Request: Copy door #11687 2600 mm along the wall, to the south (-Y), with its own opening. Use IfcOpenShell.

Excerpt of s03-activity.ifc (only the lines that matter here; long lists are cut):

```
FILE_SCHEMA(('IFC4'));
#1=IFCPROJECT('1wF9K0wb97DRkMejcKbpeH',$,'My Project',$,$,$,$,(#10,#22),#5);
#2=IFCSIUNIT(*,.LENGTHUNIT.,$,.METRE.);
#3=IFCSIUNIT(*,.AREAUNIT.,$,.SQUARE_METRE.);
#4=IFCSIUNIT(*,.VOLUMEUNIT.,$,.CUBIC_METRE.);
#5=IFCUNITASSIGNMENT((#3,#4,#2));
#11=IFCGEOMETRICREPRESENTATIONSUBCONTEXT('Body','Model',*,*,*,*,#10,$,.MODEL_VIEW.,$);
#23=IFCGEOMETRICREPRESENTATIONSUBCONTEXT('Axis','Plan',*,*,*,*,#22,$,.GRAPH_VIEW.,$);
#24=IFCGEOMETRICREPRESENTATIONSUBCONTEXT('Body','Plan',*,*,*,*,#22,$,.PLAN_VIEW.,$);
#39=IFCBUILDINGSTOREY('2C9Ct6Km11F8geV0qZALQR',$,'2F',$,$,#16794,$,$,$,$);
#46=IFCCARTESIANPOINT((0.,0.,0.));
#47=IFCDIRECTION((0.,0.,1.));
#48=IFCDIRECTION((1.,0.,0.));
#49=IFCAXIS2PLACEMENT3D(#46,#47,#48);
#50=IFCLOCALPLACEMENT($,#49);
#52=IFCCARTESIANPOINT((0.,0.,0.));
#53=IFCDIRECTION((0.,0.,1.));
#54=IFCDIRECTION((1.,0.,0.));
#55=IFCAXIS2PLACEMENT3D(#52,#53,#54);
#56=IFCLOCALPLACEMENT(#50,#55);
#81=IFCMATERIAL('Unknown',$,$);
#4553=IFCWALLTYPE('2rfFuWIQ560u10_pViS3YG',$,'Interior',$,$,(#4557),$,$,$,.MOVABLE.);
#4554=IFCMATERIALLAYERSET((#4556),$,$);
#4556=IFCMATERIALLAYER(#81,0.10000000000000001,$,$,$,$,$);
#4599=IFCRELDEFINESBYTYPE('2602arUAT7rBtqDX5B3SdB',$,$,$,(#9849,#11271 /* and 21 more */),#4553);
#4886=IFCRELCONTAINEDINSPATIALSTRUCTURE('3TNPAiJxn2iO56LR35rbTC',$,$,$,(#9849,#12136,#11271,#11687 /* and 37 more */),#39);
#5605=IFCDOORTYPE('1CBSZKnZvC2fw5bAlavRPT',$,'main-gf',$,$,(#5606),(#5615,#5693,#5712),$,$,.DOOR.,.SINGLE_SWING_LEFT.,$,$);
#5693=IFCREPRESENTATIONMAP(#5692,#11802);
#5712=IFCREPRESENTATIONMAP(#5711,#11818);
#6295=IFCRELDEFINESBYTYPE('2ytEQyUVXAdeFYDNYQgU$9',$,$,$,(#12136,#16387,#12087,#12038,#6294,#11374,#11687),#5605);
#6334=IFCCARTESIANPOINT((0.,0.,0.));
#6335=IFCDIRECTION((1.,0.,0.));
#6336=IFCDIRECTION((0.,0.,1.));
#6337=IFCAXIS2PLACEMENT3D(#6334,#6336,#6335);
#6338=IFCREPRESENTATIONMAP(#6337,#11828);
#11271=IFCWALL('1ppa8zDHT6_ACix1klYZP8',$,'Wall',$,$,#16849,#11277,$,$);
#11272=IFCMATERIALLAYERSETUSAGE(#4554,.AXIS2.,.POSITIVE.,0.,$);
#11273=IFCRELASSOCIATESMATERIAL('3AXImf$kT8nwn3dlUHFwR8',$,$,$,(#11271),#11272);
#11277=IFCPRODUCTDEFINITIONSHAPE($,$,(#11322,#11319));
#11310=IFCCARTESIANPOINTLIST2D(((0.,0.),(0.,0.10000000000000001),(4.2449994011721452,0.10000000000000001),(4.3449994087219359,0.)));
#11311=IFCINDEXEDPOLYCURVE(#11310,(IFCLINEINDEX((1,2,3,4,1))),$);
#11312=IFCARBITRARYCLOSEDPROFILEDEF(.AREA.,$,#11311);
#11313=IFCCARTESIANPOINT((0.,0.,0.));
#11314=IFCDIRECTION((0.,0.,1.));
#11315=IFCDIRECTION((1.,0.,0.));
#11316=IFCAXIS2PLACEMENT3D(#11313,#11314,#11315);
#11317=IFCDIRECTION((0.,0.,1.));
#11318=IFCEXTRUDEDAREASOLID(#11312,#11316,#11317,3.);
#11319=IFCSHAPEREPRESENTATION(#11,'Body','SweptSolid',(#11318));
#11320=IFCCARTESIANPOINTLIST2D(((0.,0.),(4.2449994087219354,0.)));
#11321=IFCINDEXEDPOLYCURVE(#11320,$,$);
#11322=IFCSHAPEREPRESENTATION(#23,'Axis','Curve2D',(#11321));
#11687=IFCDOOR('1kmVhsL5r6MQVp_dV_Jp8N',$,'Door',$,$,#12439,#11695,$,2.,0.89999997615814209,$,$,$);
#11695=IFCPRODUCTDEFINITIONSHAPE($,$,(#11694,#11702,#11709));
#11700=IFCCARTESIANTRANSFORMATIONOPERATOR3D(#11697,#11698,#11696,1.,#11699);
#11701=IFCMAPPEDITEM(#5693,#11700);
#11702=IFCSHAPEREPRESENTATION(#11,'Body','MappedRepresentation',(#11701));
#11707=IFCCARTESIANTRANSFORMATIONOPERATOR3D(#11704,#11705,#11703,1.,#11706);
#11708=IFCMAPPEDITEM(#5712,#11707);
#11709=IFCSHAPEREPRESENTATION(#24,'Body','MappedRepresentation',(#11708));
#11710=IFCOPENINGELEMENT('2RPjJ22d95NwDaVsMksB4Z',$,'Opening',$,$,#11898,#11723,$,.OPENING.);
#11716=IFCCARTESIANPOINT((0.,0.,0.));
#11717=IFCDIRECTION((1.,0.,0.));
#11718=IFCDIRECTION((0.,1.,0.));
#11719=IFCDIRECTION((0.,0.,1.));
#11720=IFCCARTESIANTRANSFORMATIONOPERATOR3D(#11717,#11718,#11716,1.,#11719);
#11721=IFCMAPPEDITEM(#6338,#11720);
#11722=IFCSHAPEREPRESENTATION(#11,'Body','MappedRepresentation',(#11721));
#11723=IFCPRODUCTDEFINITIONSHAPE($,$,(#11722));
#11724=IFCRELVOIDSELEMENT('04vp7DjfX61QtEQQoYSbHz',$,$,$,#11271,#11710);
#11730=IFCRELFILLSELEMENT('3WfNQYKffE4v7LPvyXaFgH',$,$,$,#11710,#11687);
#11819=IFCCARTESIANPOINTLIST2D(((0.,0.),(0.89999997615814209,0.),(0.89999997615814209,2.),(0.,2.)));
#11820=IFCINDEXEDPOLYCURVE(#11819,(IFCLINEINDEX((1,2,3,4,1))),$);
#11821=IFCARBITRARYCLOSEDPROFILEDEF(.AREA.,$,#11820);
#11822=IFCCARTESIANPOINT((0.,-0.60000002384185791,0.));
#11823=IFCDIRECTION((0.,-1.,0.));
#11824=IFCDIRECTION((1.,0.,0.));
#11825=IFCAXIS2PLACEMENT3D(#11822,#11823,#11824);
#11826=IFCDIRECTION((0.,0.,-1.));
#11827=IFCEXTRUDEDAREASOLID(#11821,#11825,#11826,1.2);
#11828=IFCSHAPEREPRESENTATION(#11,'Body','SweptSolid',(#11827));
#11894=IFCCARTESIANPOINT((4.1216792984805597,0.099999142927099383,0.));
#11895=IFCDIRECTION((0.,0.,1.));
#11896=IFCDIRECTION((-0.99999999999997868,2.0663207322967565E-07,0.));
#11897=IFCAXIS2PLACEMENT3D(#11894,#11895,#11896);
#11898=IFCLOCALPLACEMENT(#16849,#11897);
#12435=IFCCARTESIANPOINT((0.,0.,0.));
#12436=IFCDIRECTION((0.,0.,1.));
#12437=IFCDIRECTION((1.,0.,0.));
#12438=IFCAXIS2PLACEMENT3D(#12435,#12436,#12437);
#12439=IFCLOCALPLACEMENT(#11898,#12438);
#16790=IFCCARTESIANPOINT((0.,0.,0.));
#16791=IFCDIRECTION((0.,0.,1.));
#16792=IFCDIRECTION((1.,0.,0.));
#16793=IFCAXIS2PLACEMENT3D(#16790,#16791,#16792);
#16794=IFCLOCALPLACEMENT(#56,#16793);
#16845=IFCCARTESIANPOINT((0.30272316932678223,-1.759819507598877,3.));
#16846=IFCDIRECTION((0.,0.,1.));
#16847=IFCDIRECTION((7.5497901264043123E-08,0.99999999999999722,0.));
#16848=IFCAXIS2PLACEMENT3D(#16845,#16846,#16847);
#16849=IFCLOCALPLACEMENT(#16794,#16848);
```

```python
import ifcopenshell
import ifcopenshell.api.feature
import ifcopenshell.api.geometry
import ifcopenshell.api.root
import ifcopenshell.geom
import ifcopenshell.util.element
import ifcopenshell.util.placement
import ifcopenshell.util.shape

model = ifcopenshell.open("s03-activity.ifc")
settings = ifcopenshell.geom.settings()


def volume(element):
    """Net volume in cubic metres, openings subtracted."""
    shape = ifcopenshell.geom.create_shape(settings, element)
    return ifcopenshell.util.shape.get_volume(shape.geometry)


door = model.by_guid("1kmVhsL5r6MQVp_dV_Jp8N")
opening = door.FillsVoids[0].RelatingOpeningElement
wall = opening.VoidsElements[0].RelatingBuildingElement
before = volume(wall)
shift = ifcopenshell.util.placement.get_local_placement(wall.ObjectPlacement)[:3, 0] * -2.6

# copy_class copies the void relationship, type, container and properties, but no geometry.
new_opening = ifcopenshell.api.root.copy_class(model, product=opening)
new_opening.Representation = ifcopenshell.util.element.copy_deep(
    model, opening.Representation, exclude=["IfcGeometricRepresentationContext", "IfcRepresentationMap"]
)
new_door = ifcopenshell.api.root.copy_class(model, product=door)
new_door.Representation = ifcopenshell.util.element.copy_deep(
    model, door.Representation, exclude=["IfcGeometricRepresentationContext", "IfcRepresentationMap"]
)
ifcopenshell.api.feature.add_filling(model, opening=new_opening, element=new_door)

for old, new in ((opening, new_opening), (door, new_door)):
    matrix = ifcopenshell.util.placement.get_local_placement(old.ObjectPlacement)
    matrix[:3, 3] += shift
    ifcopenshell.api.geometry.edit_object_placement(model, product=new, matrix=matrix, is_si=False)

after = volume(wall)

print(f"wall volume {before:.3f} -> {after:.3f} m3")

model.write("s03-activity_rev.ifc")
```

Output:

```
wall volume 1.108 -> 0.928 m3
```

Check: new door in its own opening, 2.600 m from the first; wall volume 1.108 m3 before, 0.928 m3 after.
